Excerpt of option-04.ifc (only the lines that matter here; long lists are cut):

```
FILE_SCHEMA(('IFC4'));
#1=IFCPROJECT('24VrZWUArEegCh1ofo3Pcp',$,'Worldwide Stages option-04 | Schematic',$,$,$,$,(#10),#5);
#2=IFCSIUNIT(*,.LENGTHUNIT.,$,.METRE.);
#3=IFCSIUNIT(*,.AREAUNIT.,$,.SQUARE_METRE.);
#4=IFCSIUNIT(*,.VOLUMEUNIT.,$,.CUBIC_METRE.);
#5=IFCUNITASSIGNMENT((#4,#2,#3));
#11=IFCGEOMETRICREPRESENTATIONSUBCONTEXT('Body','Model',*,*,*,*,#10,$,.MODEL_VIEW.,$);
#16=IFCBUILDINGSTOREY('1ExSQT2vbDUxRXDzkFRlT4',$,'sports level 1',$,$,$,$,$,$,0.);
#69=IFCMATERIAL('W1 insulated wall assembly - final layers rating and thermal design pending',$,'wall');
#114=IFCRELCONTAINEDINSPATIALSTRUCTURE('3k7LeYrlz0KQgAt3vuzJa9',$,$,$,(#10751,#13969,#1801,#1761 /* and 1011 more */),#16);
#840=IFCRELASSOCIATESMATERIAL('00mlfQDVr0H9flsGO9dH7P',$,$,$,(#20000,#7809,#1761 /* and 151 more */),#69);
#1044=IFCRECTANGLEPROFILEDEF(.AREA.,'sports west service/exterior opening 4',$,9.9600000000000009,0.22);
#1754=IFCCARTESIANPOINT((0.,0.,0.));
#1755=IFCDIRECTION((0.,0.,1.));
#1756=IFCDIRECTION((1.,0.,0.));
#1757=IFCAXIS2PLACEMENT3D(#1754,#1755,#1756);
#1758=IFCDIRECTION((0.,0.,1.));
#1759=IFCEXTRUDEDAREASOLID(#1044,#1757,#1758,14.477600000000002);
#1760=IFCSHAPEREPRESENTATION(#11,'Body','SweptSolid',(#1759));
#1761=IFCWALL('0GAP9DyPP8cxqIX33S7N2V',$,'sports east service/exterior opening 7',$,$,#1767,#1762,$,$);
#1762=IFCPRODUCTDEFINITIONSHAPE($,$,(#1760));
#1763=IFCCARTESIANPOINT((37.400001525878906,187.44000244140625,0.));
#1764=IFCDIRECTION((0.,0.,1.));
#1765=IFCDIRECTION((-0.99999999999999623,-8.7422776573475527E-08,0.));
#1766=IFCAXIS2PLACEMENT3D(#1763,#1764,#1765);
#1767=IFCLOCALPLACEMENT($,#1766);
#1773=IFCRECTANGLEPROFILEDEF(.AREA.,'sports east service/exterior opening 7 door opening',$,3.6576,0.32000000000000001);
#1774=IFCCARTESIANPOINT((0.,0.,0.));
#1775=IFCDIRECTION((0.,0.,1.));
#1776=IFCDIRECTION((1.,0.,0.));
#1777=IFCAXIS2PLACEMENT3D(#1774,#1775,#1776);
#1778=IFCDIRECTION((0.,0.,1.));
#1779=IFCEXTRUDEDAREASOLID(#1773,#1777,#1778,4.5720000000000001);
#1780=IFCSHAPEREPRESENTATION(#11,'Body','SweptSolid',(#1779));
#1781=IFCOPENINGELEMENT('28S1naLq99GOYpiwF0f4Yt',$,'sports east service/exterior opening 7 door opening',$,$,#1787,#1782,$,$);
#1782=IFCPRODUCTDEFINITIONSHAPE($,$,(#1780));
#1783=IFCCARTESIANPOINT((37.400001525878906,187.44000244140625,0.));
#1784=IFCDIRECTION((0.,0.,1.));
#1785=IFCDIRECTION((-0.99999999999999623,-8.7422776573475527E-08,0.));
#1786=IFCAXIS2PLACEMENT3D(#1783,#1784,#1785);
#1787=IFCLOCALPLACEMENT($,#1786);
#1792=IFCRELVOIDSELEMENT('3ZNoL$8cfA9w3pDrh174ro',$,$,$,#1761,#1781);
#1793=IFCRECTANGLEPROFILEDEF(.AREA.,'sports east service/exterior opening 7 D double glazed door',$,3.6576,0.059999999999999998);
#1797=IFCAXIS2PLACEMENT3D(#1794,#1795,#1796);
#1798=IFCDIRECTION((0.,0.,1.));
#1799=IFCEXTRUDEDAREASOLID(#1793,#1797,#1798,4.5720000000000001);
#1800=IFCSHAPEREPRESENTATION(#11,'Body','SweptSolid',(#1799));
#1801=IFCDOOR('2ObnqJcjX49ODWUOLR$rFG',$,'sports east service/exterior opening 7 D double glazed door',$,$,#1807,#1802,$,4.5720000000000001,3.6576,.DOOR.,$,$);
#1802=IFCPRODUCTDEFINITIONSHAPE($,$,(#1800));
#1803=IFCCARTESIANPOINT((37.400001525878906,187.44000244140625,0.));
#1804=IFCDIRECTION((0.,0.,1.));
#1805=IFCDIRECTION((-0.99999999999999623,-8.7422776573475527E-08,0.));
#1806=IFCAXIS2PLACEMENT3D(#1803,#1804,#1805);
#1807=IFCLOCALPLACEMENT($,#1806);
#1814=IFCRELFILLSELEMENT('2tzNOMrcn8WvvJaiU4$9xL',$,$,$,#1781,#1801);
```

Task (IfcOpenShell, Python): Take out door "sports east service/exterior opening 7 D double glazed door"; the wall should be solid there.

```python
import ifcopenshell
import ifcopenshell.api.feature
import ifcopenshell.api.root
import ifcopenshell.geom
import ifcopenshell.util.shape

model = ifcopenshell.open("option-04.ifc")
settings = ifcopenshell.geom.settings()


def volume(element):
    """Net volume in cubic metres, openings subtracted."""
    shape = ifcopenshell.geom.create_shape(settings, element)
    return ifcopenshell.util.shape.get_volume(shape.geometry)


door = model.by_guid("2ObnqJcjX49ODWUOLR$rFG")
opening = door.FillsVoids[0].RelatingOpeningElement
wall = opening.VoidsElements[0].RelatingBuildingElement
before = volume(wall)

ifcopenshell.api.root.remove_product(model, product=door)
ifcopenshell.api.feature.remove_feature(model, feature=opening)

after = volume(wall)

print(f"wall volume {before:.3f} -> {after:.3f} m3")

model.write("option-04_edited.ifc")
```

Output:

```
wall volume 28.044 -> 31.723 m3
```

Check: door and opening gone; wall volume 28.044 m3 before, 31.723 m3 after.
